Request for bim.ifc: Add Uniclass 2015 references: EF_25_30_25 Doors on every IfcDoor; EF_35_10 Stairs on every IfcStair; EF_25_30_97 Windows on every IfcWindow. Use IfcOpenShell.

First a look at what the model holds.

```python
import ifcopenshell

model = ifcopenshell.open("bim.ifc")
print(model.schema)
print("classifications:", [c.Name for c in model.by_type("IfcClassification")])
for ifc_class in ("IfcDoor", "IfcRoof", "IfcStair", "IfcWall", "IfcWindow"):
    print(ifc_class, len(model.by_type(ifc_class)))
```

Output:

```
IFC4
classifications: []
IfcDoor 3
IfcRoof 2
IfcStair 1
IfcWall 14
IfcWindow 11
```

```python
import ifcopenshell
import ifcopenshell.api.classification

model = ifcopenshell.open("bim.ifc")

system = ifcopenshell.api.classification.add_classification(model, classification="Uniclass 2015")

codes = {
    "IfcDoor": ("EF_25_30_25", "Doors"),
    "IfcStair": ("EF_35_10", "Stairs"),
    "IfcWindow": ("EF_25_30_97", "Windows"),
}
for ifc_class, (code, name) in codes.items():
    products = model.by_type(ifc_class)
    ifcopenshell.api.classification.add_reference(
        model, products=products, classification=system, identification=code, name=name
    )
    print(code, len(products))

model.write("bim_v2.ifc")
```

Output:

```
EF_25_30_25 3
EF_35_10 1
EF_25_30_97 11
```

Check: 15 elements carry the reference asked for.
